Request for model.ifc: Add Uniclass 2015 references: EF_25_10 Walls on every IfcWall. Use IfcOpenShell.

First a look at what the model holds.

```python
import ifcopenshell

model = ifcopenshell.open("model.ifc")
print(model.schema)
print("classifications:", [c.Name for c in model.by_type("IfcClassification")])
for ifc_class in ("IfcDoor", "IfcRoof", "IfcStair", "IfcWall", "IfcWindow"):
    print(ifc_class, len(model.by_type(ifc_class)))
```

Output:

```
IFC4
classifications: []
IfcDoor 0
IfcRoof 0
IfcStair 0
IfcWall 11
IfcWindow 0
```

```python
import ifcopenshell
import ifcopenshell.api.classification

model = ifcopenshell.open("model.ifc")

system = ifcopenshell.api.classification.add_classification(model, classification="Uniclass 2015")

codes = {
    "IfcWall": ("EF_25_10", "Walls"),
}
for ifc_class, (code, name) in codes.items():
    products = model.by_type(ifc_class)
    ifcopenshell.api.classification.add_reference(
        model, products=products, classification=system, identification=code, name=name
    )
    print(code, len(products))

model.write("model_rev.ifc")
```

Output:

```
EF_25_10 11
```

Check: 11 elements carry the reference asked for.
